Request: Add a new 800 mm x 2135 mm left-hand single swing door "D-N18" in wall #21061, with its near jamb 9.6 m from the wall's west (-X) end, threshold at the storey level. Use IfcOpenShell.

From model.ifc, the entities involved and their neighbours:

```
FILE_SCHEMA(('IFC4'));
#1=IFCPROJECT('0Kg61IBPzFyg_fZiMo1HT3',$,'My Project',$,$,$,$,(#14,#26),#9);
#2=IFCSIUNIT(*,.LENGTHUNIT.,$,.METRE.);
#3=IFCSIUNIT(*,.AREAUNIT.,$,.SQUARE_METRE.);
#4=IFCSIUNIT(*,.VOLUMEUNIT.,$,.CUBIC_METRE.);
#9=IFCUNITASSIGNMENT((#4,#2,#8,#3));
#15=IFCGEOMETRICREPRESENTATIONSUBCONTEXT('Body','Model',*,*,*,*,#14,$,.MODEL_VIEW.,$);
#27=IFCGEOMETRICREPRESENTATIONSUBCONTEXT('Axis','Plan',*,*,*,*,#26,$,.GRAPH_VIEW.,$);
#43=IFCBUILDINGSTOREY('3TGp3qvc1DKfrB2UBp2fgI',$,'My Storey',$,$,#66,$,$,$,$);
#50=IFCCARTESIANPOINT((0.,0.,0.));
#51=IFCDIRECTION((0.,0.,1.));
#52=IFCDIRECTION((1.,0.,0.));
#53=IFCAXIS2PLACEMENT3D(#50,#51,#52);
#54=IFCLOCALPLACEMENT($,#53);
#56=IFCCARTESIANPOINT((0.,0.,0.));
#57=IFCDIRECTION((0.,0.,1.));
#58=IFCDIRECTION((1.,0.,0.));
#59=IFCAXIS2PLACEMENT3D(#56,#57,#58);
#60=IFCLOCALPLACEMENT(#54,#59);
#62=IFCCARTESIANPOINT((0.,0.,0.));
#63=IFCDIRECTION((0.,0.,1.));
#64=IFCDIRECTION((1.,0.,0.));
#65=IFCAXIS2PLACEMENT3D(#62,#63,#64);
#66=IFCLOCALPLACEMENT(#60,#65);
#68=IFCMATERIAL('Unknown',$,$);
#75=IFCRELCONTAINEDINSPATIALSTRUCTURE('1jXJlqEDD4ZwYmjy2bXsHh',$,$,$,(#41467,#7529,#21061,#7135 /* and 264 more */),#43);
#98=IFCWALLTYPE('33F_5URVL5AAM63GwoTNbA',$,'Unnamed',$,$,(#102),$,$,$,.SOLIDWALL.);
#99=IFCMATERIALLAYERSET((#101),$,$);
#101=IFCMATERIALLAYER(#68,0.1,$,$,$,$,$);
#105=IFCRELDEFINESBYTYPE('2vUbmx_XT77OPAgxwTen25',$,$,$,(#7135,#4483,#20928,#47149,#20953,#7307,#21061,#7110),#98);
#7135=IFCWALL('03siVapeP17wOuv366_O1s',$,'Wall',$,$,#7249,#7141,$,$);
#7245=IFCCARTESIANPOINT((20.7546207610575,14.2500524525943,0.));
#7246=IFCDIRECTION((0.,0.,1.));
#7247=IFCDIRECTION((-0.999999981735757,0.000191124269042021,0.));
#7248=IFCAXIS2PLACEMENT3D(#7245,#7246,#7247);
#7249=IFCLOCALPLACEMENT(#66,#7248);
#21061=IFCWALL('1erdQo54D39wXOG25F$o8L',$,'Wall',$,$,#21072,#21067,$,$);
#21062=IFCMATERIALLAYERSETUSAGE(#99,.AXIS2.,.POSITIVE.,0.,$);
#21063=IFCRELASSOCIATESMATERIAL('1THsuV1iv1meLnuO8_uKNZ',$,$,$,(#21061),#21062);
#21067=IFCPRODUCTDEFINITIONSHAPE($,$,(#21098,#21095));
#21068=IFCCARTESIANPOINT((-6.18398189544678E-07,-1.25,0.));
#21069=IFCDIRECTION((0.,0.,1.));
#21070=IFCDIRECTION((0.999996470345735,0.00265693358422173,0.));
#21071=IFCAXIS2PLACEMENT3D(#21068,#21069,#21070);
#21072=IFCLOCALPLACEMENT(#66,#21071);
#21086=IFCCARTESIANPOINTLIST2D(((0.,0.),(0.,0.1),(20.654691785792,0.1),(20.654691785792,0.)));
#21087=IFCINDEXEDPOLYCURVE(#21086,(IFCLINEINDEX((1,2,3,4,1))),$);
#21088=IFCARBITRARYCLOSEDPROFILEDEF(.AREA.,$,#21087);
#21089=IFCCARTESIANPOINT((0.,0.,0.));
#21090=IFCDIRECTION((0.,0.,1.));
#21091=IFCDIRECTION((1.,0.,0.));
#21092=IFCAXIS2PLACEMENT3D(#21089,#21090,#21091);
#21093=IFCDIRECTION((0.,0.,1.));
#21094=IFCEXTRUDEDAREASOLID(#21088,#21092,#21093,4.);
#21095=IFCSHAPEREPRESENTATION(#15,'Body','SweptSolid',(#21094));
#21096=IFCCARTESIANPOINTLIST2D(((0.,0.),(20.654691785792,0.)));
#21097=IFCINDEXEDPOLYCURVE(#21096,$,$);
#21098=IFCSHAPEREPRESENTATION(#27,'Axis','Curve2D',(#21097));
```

```python
import numpy as np
import ifcopenshell
import ifcopenshell.api.feature
import ifcopenshell.api.geometry
import ifcopenshell.api.root
import ifcopenshell.api.spatial
import ifcopenshell.geom
import ifcopenshell.util.element
import ifcopenshell.util.placement
import ifcopenshell.util.representation
import ifcopenshell.util.shape
import ifcopenshell.util.unit

model = ifcopenshell.open("model.ifc")
unit_scale = ifcopenshell.util.unit.calculate_unit_scale(model)
settings = ifcopenshell.geom.settings()


def volume(element):
    """Net volume in cubic metres, openings subtracted."""
    shape = ifcopenshell.geom.create_shape(settings, element)
    return ifcopenshell.util.shape.get_volume(shape.geometry)


wall = model.by_id(21061)
storey = ifcopenshell.util.element.get_container(wall, ifc_class="IfcBuildingStorey")
context = ifcopenshell.util.representation.get_context(model, "Model", "Body", "MODEL_VIEW")
before = volume(wall)

width, height, from_end, sill = 0.8, 2.135, 9.6, 0.0  # metres

# The wall runs along its own X axis, and the end named is its -X end.
wall_shape = ifcopenshell.geom.create_shape(settings, wall)
x, y, z = ifcopenshell.util.shape.get_vertices(wall_shape.geometry).T
start = x.min() + from_end
face, thickness = float(y.min()), float(y.max() - y.min())
wall_matrix = ifcopenshell.util.placement.get_local_placement(wall.ObjectPlacement)
level = ifcopenshell.util.placement.get_local_placement(storey.ObjectPlacement)[2, 3]


def in_wall(x, y):
    """Placement at x, y metres in the wall's axes, at sill height."""
    matrix = wall_matrix.copy()
    matrix[:, 3] = wall_matrix @ np.array([x / unit_scale, y / unit_scale, 0.0, 1.0])
    matrix[2, 3] = level + sill / unit_scale
    return matrix


# Opening: a box that overshoots both wall faces by 50 mm.
opening = ifcopenshell.api.root.create_entity(model, ifc_class="IfcOpeningElement", predefined_type="OPENING")
box = ifcopenshell.api.geometry.add_wall_representation(
    model, context=context, length=width, height=height, thickness=thickness + 0.1
)
ifcopenshell.api.geometry.assign_representation(model, product=opening, representation=box)
ifcopenshell.api.geometry.edit_object_placement(model, product=opening, matrix=in_wall(start, face - 0.05), is_si=False)
ifcopenshell.api.feature.add_feature(model, feature=opening, element=wall)

door = ifcopenshell.api.root.create_entity(model, ifc_class="IfcDoor", name="D-N18", predefined_type="DOOR")
door.OverallWidth, door.OverallHeight = width / unit_scale, height / unit_scale
door.OperationType = "SINGLE_SWING_LEFT"
body = ifcopenshell.api.geometry.add_door_representation(
    model,
    context=context,
    overall_width=door.OverallWidth,
    overall_height=door.OverallHeight,
    operation_type="SINGLE_SWING_LEFT",
    lining_properties={"LiningDepth": thickness / unit_scale, "ThresholdDepth": thickness / unit_scale},
)
ifcopenshell.api.geometry.assign_representation(model, product=door, representation=body)
ifcopenshell.api.spatial.assign_container(model, products=[door], relating_structure=storey)
ifcopenshell.api.feature.add_filling(model, opening=opening, element=door)

# The lining spans the wall, so the door starts at the wall face.
ifcopenshell.api.geometry.edit_object_placement(model, product=door, matrix=in_wall(start, face), is_si=False)

after = volume(wall)

print(f"wall volume {before:.3f} -> {after:.3f} m3")

model.write("model-out.ifc")
```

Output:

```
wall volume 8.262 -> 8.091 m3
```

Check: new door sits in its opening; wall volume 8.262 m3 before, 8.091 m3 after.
